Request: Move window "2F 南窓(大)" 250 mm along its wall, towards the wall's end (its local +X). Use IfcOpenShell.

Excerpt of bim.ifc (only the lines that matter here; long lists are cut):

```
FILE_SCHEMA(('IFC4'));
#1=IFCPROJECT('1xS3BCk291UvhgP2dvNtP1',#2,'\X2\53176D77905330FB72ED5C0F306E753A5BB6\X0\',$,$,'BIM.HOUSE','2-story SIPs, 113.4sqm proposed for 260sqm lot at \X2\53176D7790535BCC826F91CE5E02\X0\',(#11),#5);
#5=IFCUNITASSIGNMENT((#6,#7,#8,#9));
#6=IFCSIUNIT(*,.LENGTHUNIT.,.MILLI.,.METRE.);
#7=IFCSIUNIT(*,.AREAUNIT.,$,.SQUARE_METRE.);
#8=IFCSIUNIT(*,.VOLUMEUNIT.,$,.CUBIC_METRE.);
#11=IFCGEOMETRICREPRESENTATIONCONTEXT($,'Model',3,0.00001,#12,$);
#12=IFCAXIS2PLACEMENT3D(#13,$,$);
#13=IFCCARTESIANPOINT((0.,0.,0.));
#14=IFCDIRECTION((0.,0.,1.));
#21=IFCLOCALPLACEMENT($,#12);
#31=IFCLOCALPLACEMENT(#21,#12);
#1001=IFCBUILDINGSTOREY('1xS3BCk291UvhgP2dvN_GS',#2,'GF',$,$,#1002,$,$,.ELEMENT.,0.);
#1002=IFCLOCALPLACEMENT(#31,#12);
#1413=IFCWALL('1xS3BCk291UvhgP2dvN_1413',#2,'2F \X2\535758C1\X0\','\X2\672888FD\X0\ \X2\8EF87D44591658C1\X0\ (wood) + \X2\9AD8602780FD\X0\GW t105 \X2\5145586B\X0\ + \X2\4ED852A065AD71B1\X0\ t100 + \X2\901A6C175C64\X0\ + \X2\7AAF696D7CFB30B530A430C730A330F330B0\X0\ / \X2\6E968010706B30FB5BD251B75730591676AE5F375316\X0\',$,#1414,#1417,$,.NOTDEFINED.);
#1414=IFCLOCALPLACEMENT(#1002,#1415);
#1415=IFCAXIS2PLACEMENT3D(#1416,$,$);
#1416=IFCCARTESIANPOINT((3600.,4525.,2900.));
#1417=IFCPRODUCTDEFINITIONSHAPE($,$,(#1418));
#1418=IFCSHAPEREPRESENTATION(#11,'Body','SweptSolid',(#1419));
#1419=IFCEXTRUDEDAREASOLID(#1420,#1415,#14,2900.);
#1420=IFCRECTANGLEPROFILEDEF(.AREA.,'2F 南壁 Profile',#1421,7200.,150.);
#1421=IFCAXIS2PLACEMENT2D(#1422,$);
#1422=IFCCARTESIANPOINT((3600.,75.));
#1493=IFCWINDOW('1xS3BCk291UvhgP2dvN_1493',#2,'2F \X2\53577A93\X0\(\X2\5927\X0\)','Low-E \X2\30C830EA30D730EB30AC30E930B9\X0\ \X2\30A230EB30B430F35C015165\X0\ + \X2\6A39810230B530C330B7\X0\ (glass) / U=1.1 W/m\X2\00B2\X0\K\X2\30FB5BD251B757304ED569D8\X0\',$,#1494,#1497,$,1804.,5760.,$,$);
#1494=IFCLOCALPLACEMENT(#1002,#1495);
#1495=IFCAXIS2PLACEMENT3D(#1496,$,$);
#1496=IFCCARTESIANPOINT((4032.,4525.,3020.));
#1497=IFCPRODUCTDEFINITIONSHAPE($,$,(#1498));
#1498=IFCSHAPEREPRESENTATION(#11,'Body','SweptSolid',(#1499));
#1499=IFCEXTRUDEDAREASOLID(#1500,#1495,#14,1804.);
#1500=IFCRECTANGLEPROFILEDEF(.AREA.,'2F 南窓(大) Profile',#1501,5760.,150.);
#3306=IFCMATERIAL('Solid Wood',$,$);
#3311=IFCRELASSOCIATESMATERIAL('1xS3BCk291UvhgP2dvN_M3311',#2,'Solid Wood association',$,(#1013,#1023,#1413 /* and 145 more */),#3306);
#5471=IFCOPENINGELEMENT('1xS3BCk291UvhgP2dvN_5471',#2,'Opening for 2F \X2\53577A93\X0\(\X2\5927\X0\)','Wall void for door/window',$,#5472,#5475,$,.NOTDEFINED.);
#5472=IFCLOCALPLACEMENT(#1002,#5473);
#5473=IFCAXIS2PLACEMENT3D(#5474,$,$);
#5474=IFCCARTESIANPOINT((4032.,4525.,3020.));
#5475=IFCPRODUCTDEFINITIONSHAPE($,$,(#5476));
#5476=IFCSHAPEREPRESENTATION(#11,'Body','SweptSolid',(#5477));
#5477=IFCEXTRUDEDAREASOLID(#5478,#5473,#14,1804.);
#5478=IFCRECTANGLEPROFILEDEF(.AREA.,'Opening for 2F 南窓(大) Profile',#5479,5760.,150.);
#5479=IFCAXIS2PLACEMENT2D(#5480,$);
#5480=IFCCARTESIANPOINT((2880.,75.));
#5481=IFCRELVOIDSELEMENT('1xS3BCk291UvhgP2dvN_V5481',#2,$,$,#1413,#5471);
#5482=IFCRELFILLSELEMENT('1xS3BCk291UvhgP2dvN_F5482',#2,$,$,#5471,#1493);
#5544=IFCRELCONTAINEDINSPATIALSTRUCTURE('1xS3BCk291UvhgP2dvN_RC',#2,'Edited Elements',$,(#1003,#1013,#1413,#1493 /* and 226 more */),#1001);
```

```python
import ifcopenshell
import ifcopenshell.api.geometry
import ifcopenshell.util.placement
import ifcopenshell.util.unit

model = ifcopenshell.open("bim.ifc")
unit_scale = ifcopenshell.util.unit.calculate_unit_scale(model)

window = model.by_guid("1xS3BCk291UvhgP2dvN_1493")
opening = window.FillsVoids[0].RelatingOpeningElement
wall = opening.VoidsElements[0].RelatingBuildingElement

wall_matrix = ifcopenshell.util.placement.get_local_placement(wall.ObjectPlacement)
shift = wall_matrix[:3, 0] * 0.25 / unit_scale
before = ifcopenshell.util.placement.get_local_placement(window.ObjectPlacement)[:3, 3].copy()

# The window is not placed relative to its opening, so move both.
for product in (opening, window):
    matrix = ifcopenshell.util.placement.get_local_placement(product.ObjectPlacement)
    matrix[:3, 3] += shift
    ifcopenshell.api.geometry.edit_object_placement(model, product=product, matrix=matrix, is_si=False)

after = ifcopenshell.util.placement.get_local_placement(window.ObjectPlacement)[:3, 3]
print("window moved by", (after - before).round(3) + 0.0)

model.write("bim_v2.ifc")
```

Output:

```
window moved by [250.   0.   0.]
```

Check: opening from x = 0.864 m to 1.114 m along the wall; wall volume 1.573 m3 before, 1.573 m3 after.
